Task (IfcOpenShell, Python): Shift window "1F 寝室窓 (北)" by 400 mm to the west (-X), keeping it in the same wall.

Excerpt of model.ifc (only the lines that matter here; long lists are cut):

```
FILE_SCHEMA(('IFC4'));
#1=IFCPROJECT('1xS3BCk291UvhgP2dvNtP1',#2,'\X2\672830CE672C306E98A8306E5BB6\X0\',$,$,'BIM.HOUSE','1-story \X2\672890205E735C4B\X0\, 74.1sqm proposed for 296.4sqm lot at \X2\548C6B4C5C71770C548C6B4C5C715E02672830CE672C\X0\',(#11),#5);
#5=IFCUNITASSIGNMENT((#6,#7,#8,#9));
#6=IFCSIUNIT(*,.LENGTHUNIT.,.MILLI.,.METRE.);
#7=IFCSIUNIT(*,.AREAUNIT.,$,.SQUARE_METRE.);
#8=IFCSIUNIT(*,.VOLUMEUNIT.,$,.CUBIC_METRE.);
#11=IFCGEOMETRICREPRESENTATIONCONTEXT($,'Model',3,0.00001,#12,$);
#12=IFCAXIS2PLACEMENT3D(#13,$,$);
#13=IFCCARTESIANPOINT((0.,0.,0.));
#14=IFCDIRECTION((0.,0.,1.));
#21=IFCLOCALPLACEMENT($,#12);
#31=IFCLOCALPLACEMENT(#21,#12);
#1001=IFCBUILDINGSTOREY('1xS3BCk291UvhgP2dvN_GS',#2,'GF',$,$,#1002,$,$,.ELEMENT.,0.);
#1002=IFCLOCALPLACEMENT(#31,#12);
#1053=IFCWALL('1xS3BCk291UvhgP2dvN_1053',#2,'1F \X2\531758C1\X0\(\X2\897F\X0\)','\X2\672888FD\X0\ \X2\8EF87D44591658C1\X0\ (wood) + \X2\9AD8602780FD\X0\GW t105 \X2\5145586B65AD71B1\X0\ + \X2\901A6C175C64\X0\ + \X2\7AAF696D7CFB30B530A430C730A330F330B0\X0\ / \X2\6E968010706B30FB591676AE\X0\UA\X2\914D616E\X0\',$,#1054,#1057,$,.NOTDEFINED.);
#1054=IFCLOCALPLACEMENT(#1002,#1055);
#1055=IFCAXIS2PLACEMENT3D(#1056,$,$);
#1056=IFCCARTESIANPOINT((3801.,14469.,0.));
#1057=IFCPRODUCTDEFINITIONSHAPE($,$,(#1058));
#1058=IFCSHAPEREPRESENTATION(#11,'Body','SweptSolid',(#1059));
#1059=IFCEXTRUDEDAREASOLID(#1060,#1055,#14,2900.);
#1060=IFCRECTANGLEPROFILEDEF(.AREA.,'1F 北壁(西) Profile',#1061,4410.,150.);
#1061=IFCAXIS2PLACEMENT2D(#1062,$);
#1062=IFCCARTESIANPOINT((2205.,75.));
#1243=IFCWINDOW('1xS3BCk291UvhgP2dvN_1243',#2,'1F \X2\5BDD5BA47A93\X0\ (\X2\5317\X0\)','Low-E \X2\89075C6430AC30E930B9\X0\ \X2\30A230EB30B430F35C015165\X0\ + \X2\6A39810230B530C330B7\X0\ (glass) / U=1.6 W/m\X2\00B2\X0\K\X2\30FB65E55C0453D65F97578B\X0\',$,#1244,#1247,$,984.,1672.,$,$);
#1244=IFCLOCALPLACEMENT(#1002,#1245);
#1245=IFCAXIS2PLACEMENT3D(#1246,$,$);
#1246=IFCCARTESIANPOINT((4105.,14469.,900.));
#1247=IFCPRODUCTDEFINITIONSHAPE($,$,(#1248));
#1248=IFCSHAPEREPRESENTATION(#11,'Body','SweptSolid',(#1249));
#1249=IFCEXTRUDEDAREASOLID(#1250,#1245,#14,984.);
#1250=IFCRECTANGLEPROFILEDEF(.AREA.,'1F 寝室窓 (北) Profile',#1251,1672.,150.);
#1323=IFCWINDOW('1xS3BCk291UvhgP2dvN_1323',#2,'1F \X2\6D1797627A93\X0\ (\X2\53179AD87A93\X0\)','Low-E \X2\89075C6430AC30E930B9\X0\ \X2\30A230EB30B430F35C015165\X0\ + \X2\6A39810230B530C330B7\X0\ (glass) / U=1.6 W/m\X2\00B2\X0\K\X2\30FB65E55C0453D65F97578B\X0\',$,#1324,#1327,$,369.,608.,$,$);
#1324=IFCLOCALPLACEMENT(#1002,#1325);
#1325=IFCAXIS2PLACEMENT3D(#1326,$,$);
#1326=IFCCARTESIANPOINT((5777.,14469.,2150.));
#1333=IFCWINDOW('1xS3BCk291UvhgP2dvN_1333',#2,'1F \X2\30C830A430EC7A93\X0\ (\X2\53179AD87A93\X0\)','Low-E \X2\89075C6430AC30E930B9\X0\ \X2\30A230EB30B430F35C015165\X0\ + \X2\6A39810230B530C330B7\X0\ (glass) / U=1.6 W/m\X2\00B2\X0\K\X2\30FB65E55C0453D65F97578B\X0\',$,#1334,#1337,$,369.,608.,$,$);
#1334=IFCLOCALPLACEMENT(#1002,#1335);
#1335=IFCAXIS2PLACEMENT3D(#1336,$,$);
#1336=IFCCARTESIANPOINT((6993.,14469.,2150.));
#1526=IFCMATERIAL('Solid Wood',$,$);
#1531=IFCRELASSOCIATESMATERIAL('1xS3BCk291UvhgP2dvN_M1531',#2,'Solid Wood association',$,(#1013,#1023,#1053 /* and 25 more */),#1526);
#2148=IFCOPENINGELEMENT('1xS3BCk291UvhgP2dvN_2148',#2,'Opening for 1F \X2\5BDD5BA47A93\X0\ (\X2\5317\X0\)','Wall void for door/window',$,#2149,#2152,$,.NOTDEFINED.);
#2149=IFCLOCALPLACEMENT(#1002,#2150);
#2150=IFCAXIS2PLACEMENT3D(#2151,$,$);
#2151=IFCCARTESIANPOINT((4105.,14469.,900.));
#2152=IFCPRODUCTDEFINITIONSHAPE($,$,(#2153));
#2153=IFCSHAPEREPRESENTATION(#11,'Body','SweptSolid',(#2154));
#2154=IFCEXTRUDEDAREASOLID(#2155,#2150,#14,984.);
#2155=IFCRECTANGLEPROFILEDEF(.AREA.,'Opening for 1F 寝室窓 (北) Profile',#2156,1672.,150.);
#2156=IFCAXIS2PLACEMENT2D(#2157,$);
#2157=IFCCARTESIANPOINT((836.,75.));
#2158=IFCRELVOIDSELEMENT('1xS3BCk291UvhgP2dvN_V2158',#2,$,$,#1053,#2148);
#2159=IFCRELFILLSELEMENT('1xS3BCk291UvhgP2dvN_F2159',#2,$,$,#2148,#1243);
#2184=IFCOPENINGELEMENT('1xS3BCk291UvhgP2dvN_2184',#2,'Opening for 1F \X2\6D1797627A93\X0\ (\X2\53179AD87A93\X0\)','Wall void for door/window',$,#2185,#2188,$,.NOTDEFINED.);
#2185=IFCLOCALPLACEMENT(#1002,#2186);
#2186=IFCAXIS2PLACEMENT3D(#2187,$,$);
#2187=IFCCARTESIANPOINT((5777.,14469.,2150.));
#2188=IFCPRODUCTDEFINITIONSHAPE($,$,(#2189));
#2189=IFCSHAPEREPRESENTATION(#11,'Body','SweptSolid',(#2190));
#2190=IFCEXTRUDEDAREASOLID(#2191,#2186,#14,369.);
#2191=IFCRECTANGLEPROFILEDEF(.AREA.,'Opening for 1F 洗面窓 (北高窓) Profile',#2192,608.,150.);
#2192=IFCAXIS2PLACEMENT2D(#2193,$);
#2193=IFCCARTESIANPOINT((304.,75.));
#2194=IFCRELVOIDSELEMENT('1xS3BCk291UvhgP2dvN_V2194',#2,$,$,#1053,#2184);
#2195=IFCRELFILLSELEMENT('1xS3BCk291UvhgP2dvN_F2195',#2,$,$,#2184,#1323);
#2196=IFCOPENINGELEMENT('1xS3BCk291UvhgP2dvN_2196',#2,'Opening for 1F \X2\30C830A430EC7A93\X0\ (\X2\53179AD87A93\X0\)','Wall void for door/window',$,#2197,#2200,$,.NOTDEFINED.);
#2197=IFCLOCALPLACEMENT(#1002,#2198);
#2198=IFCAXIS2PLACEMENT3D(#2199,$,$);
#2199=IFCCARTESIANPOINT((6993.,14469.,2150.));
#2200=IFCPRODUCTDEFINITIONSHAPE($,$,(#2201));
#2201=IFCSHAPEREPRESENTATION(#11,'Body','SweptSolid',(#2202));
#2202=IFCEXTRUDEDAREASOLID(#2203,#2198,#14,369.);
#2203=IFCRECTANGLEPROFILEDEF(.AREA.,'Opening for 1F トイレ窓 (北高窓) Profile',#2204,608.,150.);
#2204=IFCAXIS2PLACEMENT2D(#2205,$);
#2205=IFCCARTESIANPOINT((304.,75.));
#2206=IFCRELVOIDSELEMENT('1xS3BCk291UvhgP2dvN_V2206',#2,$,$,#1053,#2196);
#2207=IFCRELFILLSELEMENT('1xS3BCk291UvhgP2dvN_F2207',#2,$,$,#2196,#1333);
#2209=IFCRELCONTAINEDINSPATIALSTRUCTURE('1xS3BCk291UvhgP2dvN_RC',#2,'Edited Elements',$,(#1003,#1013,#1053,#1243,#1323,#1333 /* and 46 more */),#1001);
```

```python
import ifcopenshell
import ifcopenshell.api.geometry
import ifcopenshell.util.placement
import ifcopenshell.util.unit

model = ifcopenshell.open("model.ifc")
unit_scale = ifcopenshell.util.unit.calculate_unit_scale(model)

window = model.by_guid("1xS3BCk291UvhgP2dvN_1243")
opening = window.FillsVoids[0].RelatingOpeningElement
wall = opening.VoidsElements[0].RelatingBuildingElement

wall_matrix = ifcopenshell.util.placement.get_local_placement(wall.ObjectPlacement)
shift = wall_matrix[:3, 0] * -0.4 / unit_scale
before = ifcopenshell.util.placement.get_local_placement(window.ObjectPlacement)[:3, 3].copy()

# The window is not placed relative to its opening, so move both.
for product in (opening, window):
    matrix = ifcopenshell.util.placement.get_local_placement(product.ObjectPlacement)
    matrix[:3, 3] += shift
    ifcopenshell.api.geometry.edit_object_placement(model, product=product, matrix=matrix, is_si=False)

after = ifcopenshell.util.placement.get_local_placement(window.ObjectPlacement)[:3, 3]
print("window moved by", (after - before).round(3) + 0.0)

model.write("model_updated.ifc")
```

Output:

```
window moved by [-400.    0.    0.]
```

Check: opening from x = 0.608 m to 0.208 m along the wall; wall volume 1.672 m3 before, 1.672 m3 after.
